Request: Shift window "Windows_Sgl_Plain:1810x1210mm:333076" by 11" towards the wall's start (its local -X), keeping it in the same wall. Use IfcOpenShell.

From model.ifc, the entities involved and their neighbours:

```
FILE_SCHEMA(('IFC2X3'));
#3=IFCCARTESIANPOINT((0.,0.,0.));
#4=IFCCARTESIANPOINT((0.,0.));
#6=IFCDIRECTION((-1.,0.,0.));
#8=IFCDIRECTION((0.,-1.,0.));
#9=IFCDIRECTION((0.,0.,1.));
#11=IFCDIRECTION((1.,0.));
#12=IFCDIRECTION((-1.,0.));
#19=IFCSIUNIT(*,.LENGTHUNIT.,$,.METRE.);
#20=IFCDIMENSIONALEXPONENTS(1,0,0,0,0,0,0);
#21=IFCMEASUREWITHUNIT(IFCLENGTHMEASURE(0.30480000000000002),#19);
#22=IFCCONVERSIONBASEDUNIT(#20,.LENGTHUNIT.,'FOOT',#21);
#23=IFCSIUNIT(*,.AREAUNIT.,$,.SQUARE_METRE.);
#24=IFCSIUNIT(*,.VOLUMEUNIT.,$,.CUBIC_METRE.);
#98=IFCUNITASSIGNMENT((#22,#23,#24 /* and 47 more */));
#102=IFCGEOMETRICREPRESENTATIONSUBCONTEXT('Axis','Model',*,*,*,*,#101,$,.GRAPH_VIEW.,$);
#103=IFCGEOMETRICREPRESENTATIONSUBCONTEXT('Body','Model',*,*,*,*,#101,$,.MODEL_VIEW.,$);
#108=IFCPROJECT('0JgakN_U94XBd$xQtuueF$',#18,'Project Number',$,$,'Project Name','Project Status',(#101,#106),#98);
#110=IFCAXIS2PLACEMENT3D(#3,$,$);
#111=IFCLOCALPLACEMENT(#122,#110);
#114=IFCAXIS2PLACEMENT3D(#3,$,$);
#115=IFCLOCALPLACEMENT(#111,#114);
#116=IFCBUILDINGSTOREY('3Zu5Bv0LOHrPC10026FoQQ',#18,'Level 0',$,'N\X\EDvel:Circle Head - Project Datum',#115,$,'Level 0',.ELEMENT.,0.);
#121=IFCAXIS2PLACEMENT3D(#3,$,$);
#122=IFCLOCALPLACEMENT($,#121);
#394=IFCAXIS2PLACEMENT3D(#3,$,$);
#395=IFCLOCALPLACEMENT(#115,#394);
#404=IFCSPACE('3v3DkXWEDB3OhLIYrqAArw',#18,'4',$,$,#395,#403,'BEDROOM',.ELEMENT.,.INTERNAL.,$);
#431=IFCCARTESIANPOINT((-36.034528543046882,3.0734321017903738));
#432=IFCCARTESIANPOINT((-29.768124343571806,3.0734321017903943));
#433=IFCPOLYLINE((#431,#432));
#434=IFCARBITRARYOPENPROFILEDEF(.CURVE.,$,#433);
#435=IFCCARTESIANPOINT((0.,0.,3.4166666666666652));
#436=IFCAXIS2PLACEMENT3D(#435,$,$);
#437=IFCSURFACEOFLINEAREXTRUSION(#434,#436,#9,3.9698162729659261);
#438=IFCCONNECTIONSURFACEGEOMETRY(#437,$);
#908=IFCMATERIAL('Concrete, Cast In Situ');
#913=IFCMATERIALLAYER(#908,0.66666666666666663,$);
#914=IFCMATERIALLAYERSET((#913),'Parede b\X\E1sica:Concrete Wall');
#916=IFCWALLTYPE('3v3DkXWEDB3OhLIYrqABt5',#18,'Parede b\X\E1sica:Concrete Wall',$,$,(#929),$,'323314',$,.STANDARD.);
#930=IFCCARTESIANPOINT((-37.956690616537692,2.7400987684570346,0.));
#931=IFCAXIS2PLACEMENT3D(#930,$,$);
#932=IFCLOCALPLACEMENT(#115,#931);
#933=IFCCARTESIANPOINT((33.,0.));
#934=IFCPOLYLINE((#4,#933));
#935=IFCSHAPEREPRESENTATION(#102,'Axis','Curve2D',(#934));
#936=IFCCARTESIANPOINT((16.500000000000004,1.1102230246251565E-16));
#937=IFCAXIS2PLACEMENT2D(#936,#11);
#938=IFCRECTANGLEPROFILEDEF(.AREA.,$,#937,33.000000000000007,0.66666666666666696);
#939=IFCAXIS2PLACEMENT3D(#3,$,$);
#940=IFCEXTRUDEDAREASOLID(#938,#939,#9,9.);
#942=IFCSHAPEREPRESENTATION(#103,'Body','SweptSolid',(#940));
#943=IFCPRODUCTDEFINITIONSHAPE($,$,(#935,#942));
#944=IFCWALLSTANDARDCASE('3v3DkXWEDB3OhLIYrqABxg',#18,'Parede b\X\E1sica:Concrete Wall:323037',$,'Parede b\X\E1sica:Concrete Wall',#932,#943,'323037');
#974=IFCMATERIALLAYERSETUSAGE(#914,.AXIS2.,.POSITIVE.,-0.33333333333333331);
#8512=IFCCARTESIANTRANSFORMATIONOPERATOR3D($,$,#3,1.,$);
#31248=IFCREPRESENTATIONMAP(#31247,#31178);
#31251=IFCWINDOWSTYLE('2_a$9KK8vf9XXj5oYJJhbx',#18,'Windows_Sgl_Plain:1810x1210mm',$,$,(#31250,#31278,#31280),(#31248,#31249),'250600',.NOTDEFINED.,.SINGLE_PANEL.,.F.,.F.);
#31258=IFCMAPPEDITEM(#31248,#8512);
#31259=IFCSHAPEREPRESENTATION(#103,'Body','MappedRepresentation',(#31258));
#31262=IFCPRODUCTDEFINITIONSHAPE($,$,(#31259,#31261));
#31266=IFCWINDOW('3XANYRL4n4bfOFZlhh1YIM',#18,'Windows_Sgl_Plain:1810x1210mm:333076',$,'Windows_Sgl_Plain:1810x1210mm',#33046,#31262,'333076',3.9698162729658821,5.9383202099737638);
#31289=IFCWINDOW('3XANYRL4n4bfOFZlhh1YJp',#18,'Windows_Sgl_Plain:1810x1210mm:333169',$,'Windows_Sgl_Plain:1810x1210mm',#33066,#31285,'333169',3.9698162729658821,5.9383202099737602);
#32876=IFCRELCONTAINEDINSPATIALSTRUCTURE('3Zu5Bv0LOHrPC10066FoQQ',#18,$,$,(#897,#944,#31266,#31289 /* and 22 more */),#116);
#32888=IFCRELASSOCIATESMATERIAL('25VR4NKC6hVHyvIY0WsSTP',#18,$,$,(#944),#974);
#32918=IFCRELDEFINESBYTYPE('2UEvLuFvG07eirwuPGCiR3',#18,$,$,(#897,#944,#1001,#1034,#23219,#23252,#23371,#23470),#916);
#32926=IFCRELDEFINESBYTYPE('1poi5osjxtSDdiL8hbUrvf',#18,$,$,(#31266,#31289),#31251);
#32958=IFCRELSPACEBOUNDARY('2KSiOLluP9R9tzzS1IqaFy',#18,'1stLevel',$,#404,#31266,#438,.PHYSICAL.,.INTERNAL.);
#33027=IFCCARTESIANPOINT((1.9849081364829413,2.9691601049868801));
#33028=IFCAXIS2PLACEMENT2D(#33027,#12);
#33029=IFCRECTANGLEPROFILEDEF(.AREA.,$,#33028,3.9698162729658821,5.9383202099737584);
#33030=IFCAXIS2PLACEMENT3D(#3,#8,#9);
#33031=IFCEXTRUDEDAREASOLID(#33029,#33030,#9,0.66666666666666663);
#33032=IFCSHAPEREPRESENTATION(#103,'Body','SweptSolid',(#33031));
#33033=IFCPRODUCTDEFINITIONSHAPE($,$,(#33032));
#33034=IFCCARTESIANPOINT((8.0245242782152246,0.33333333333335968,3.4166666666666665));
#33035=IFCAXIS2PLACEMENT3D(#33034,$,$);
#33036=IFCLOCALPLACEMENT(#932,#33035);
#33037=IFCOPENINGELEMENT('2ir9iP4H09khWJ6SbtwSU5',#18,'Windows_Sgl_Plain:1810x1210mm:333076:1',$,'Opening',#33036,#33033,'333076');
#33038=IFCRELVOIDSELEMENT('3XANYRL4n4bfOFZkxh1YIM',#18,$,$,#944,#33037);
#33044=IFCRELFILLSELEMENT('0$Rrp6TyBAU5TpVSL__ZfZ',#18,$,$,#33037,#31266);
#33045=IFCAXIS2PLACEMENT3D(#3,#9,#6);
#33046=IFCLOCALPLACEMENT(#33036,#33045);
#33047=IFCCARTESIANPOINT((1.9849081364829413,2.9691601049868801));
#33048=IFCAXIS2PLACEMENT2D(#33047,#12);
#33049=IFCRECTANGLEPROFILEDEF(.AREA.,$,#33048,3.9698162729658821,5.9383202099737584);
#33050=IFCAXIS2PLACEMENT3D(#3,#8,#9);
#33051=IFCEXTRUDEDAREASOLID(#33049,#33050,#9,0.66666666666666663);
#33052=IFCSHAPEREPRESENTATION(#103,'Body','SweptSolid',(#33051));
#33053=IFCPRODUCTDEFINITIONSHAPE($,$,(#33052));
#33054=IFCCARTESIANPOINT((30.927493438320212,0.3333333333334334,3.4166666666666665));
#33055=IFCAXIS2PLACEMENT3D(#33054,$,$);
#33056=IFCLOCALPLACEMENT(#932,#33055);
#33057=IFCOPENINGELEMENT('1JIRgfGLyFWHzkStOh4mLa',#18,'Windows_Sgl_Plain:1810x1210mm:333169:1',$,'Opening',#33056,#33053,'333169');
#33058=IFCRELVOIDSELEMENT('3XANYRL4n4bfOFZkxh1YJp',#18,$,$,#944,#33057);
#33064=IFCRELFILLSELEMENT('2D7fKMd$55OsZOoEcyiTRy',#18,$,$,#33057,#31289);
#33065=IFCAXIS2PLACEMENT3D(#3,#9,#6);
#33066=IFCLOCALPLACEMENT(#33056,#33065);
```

```python
import numpy as np
import ifcopenshell
import ifcopenshell.api.geometry
import ifcopenshell.util.placement
import ifcopenshell.util.unit

model = ifcopenshell.open("model.ifc")
unit_scale = ifcopenshell.util.unit.calculate_unit_scale(model)

window = model.by_id(31266)
opening = window.FillsVoids[0].RelatingOpeningElement
wall = opening.VoidsElements[0].RelatingBuildingElement

wall_matrix = ifcopenshell.util.placement.get_local_placement(wall.ObjectPlacement)
shift = wall_matrix[:3, 0] * -11 * 0.0254 / unit_scale
before = ifcopenshell.util.placement.get_local_placement(window.ObjectPlacement)[:3, 3].copy()

# The window is placed relative to its opening, so it follows when the opening moves.
matrix = ifcopenshell.util.placement.get_local_placement(opening.ObjectPlacement)
matrix[:3, 3] += shift
ifcopenshell.api.geometry.edit_object_placement(
    model, product=opening, matrix=matrix, is_si=False, should_transform_children=True
)

# Space boundary surfaces are stored in each space's coordinates; move them too.
for rel in window.ProvidesBoundaries:
    if not rel.ConnectionGeometry:
        continue
    surface = rel.ConnectionGeometry.SurfaceOnRelatingElement
    space_matrix = ifcopenshell.util.placement.get_local_placement(rel.RelatingSpace.ObjectPlacement)
    point = np.array(surface.Position.Location.Coordinates) + space_matrix[:3, :3].T @ shift
    surface.Position = model.createIfcAxis2Placement3D(
        model.createIfcCartesianPoint(point.tolist()), surface.Position.Axis, surface.Position.RefDirection
    )

after = ifcopenshell.util.placement.get_local_placement(window.ObjectPlacement)[:3, 3]
print("window moved by", (after - before).round(3) + 0.0)

model.write("model_rev.ifc")
```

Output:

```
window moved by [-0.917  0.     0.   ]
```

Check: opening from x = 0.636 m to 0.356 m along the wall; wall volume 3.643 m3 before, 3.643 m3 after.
